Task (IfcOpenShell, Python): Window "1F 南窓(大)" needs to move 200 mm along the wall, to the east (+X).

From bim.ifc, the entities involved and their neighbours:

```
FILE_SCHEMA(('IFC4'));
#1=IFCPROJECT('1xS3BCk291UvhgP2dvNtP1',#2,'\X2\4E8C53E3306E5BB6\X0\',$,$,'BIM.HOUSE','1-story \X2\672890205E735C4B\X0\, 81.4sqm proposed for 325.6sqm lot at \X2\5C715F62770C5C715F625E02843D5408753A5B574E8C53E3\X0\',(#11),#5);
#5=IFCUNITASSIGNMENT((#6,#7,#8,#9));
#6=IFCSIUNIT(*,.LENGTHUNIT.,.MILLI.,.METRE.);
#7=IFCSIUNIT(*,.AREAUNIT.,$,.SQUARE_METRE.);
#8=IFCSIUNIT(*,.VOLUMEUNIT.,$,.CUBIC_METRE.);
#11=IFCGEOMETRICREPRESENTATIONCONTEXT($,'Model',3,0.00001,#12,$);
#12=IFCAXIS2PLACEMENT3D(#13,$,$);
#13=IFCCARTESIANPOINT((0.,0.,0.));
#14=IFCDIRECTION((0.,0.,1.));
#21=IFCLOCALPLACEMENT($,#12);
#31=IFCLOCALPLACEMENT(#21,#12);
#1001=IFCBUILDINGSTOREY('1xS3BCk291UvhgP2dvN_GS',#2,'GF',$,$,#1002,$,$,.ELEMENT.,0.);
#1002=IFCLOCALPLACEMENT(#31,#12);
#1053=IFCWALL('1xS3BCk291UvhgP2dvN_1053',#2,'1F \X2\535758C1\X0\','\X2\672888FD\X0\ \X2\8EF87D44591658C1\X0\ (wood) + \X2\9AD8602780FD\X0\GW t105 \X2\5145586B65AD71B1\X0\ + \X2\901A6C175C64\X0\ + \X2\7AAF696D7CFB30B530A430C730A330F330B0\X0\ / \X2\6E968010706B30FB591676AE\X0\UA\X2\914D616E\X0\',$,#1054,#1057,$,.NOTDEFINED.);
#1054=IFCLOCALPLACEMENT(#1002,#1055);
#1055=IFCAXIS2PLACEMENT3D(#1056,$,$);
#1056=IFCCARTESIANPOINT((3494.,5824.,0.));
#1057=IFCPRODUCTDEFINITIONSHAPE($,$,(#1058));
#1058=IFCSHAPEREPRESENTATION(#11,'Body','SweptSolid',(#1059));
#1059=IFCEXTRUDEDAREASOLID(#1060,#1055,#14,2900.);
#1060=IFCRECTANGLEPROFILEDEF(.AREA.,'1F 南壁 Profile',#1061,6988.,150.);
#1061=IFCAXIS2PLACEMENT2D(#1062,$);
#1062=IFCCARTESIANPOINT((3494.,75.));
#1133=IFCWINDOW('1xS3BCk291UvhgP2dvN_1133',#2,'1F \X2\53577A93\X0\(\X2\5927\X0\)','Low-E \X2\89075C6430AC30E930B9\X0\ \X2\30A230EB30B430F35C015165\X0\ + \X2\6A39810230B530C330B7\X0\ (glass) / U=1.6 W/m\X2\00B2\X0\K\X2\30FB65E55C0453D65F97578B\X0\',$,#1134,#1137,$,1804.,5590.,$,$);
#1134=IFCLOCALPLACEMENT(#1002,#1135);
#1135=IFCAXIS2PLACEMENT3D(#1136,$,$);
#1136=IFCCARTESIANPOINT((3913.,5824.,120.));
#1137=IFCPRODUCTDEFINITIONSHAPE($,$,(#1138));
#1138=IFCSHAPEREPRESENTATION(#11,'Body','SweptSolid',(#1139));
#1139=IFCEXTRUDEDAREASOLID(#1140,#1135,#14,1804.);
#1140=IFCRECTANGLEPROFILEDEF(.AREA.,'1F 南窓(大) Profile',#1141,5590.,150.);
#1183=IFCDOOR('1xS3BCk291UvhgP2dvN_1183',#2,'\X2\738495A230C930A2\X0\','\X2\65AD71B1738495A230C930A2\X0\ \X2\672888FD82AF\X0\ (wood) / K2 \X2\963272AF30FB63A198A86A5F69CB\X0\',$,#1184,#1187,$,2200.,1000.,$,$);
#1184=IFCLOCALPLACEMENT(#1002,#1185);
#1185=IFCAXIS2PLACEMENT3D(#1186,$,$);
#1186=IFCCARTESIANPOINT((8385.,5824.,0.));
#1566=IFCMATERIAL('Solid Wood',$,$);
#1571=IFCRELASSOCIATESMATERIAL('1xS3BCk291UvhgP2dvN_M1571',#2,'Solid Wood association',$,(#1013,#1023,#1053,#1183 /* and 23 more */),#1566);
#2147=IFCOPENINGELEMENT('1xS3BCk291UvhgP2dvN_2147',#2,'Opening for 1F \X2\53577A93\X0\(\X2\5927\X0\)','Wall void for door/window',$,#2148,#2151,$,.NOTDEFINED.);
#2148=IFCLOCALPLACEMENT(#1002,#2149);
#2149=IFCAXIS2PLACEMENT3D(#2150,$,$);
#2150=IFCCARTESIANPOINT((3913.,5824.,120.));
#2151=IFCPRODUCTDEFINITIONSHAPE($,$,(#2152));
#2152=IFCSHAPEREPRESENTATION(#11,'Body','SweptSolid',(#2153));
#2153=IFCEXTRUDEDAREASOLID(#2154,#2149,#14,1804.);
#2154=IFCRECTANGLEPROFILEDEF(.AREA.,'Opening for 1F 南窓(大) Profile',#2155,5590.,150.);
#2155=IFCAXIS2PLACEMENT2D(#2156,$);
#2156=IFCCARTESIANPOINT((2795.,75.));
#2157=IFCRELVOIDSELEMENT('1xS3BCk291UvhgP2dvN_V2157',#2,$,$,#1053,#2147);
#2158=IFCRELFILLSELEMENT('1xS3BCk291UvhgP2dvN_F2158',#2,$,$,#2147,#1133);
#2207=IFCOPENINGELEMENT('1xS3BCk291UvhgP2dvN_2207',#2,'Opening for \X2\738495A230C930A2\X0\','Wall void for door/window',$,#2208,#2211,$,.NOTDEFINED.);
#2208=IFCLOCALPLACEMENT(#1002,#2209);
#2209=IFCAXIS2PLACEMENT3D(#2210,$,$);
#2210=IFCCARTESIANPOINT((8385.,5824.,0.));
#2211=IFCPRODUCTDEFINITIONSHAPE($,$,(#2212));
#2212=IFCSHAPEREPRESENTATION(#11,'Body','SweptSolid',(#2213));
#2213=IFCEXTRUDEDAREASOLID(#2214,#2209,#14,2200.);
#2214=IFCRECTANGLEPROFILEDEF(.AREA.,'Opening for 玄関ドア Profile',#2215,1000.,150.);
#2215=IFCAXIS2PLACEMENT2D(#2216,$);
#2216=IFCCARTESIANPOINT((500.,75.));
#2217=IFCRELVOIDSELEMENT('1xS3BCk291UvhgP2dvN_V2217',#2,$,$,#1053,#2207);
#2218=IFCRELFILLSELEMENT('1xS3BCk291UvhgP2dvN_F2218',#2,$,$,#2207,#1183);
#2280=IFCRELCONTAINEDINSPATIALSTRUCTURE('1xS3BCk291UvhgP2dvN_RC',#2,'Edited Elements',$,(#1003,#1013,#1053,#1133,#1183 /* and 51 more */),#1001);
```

```python
import ifcopenshell
import ifcopenshell.api.geometry
import ifcopenshell.util.placement
import ifcopenshell.util.unit

model = ifcopenshell.open("bim.ifc")
unit_scale = ifcopenshell.util.unit.calculate_unit_scale(model)

window = model.by_id(1133)
opening = window.FillsVoids[0].RelatingOpeningElement
wall = opening.VoidsElements[0].RelatingBuildingElement

wall_matrix = ifcopenshell.util.placement.get_local_placement(wall.ObjectPlacement)
shift = wall_matrix[:3, 0] * 0.2 / unit_scale
before = ifcopenshell.util.placement.get_local_placement(window.ObjectPlacement)[:3, 3].copy()

# The window is not placed relative to its opening, so move both.
for product in (opening, window):
    matrix = ifcopenshell.util.placement.get_local_placement(product.ObjectPlacement)
    matrix[:3, 3] += shift
    ifcopenshell.api.geometry.edit_object_placement(model, product=product, matrix=matrix, is_si=False)

after = ifcopenshell.util.placement.get_local_placement(window.ObjectPlacement)[:3, 3]
print("window moved by", (after - before).round(3) + 0.0)

model.write("bim_rev.ifc")
```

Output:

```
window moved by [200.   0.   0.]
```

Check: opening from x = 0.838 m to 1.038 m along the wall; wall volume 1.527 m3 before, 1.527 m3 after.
